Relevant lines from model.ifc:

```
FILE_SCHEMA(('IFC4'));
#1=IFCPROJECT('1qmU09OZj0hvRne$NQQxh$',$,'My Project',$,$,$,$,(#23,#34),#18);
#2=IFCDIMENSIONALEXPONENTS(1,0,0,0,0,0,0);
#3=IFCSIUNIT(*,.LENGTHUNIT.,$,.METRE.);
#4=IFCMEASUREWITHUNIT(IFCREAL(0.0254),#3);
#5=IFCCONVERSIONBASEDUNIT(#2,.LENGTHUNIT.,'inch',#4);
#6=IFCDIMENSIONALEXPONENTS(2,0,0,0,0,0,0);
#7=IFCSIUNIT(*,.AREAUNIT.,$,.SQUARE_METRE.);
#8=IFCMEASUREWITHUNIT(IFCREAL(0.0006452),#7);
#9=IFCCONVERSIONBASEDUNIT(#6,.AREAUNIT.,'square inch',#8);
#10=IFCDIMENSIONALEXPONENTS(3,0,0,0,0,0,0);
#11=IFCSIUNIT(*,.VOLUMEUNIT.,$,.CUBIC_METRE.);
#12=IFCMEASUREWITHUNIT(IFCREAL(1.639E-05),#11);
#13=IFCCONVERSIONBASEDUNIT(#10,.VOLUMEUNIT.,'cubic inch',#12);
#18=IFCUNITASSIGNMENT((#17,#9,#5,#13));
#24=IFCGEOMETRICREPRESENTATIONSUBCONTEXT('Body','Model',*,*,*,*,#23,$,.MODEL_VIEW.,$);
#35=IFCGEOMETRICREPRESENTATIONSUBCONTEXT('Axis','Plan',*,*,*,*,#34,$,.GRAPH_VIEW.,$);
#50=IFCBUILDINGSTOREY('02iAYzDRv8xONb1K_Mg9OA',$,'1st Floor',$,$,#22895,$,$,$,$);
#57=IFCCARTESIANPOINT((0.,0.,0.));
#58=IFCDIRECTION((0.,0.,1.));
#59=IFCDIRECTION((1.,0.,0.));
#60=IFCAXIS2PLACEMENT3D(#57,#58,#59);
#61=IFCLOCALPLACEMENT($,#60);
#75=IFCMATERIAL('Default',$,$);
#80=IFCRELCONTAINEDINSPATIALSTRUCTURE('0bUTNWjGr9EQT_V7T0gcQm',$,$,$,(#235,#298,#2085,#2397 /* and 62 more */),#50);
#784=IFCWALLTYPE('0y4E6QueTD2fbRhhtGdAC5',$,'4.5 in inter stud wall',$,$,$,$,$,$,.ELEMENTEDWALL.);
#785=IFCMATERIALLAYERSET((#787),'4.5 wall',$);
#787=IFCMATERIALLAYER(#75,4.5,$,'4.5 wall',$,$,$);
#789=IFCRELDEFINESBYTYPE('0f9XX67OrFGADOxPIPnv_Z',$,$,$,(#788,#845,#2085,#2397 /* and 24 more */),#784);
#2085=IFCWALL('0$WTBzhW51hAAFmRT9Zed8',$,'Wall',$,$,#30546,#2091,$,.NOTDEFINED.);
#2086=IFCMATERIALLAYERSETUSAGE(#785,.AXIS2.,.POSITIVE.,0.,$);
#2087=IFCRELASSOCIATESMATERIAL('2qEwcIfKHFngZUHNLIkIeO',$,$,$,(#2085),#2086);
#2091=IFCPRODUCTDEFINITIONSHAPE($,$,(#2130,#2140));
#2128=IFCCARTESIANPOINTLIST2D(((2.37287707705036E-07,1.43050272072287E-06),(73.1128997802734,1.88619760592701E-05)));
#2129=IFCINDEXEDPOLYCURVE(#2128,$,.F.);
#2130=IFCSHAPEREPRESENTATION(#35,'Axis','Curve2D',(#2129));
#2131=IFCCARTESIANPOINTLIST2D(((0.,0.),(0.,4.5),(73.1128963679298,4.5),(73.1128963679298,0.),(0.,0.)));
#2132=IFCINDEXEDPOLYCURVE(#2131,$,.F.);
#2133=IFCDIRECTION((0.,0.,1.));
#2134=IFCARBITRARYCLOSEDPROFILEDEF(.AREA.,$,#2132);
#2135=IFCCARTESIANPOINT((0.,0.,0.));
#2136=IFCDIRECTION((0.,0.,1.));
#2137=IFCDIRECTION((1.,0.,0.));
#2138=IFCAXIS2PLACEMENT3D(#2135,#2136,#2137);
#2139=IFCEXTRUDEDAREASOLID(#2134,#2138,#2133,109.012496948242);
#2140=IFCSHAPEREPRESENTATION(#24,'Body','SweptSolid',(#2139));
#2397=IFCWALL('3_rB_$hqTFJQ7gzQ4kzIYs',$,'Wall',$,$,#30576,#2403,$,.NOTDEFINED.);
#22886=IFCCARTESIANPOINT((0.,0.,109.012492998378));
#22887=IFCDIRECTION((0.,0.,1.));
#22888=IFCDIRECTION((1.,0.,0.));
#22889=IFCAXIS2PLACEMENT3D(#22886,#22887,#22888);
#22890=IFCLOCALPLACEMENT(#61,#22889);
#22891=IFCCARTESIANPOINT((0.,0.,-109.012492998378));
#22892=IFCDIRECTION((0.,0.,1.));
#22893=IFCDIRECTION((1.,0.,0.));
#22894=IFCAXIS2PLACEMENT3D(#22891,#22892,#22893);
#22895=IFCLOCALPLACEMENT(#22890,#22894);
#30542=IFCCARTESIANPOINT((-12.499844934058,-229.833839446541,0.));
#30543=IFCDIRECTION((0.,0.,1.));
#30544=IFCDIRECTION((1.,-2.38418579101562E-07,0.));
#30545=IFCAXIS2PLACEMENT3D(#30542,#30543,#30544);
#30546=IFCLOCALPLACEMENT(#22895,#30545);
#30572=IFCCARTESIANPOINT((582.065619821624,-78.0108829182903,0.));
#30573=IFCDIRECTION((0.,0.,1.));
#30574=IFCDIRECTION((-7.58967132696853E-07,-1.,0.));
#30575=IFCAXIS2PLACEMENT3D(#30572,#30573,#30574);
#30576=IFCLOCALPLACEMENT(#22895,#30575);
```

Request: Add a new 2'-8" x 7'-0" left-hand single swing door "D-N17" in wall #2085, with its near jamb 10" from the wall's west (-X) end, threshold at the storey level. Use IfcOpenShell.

```python
import numpy as np
import ifcopenshell
import ifcopenshell.api.feature
import ifcopenshell.api.geometry
import ifcopenshell.api.root
import ifcopenshell.api.spatial
import ifcopenshell.geom
import ifcopenshell.util.element
import ifcopenshell.util.placement
import ifcopenshell.util.representation
import ifcopenshell.util.shape
import ifcopenshell.util.unit

model = ifcopenshell.open("model.ifc")
unit_scale = ifcopenshell.util.unit.calculate_unit_scale(model)
settings = ifcopenshell.geom.settings()


def volume(element):
    """Net volume in cubic metres, openings subtracted."""
    shape = ifcopenshell.geom.create_shape(settings, element)
    return ifcopenshell.util.shape.get_volume(shape.geometry)


wall = model.by_guid("0$WTBzhW51hAAFmRT9Zed8")
storey = ifcopenshell.util.element.get_container(wall, ifc_class="IfcBuildingStorey")
context = ifcopenshell.util.representation.get_context(model, "Model", "Body", "MODEL_VIEW")
before = volume(wall)

width, height, from_end, sill = 0.8128, 2.1336, 0.254, 0.0  # metres

# The wall runs along its own X axis, and the end named is its -X end.
wall_shape = ifcopenshell.geom.create_shape(settings, wall)
x, y, z = ifcopenshell.util.shape.get_vertices(wall_shape.geometry).T
start = x.min() + from_end
face, thickness = float(y.min()), float(y.max() - y.min())
wall_matrix = ifcopenshell.util.placement.get_local_placement(wall.ObjectPlacement)
level = ifcopenshell.util.placement.get_local_placement(storey.ObjectPlacement)[2, 3]


def in_wall(x, y):
    """Placement at x, y metres in the wall's axes, at sill height."""
    matrix = wall_matrix.copy()
    matrix[:, 3] = wall_matrix @ np.array([x / unit_scale, y / unit_scale, 0.0, 1.0])
    matrix[2, 3] = level + sill / unit_scale
    return matrix


# Opening: a box that overshoots both wall faces by 50 mm.
opening = ifcopenshell.api.root.create_entity(model, ifc_class="IfcOpeningElement", predefined_type="OPENING")
box = ifcopenshell.api.geometry.add_wall_representation(
    model, context=context, length=width, height=height, thickness=thickness + 0.1
)
ifcopenshell.api.geometry.assign_representation(model, product=opening, representation=box)
ifcopenshell.api.geometry.edit_object_placement(model, product=opening, matrix=in_wall(start, face - 0.05), is_si=False)
ifcopenshell.api.feature.add_feature(model, feature=opening, element=wall)

door = ifcopenshell.api.root.create_entity(model, ifc_class="IfcDoor", name="D-N17", predefined_type="DOOR")
door.OverallWidth, door.OverallHeight = width / unit_scale, height / unit_scale
door.OperationType = "SINGLE_SWING_LEFT"
body = ifcopenshell.api.geometry.add_door_representation(
    model,
    context=context,
    overall_width=door.OverallWidth,
    overall_height=door.OverallHeight,
    operation_type="SINGLE_SWING_LEFT",
    lining_properties={"LiningDepth": thickness / unit_scale, "ThresholdDepth": thickness / unit_scale},
)
ifcopenshell.api.geometry.assign_representation(model, product=door, representation=body)
ifcopenshell.api.spatial.assign_container(model, products=[door], relating_structure=storey)
ifcopenshell.api.feature.add_filling(model, opening=opening, element=door)

# The lining spans the wall, so the door starts at the wall face.
ifcopenshell.api.geometry.edit_object_placement(model, product=door, matrix=in_wall(start, face), is_si=False)

after = volume(wall)

print(f"wall volume {before:.3f} -> {after:.3f} m3")

model.write("model_rev.ifc")
```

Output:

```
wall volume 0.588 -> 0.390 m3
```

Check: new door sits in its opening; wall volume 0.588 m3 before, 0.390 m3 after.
